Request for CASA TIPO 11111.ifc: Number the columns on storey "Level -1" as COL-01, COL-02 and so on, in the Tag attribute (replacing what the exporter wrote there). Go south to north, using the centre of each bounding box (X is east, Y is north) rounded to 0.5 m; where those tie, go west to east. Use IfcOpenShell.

First a look at what the model holds.

```python
import ifcopenshell
import ifcopenshell.util.element
import ifcopenshell.util.placement

model = ifcopenshell.open("CASA TIPO 11111.ifc")
print(model.schema)
storey = next(s for s in model.by_type("IfcBuildingStorey") if s.Name == "Level -1")
columns = [e for e in ifcopenshell.util.element.get_decomposition(storey) if e.is_a("IfcColumn")]
for e in sorted(columns, key=lambda e: e.id()):
    origin = ifcopenshell.util.placement.get_local_placement(e.ObjectPlacement)[:3, 3]
    print(e.id(), e.Tag, e.Name, origin.round(2) + 0.0, sep=" | ")
```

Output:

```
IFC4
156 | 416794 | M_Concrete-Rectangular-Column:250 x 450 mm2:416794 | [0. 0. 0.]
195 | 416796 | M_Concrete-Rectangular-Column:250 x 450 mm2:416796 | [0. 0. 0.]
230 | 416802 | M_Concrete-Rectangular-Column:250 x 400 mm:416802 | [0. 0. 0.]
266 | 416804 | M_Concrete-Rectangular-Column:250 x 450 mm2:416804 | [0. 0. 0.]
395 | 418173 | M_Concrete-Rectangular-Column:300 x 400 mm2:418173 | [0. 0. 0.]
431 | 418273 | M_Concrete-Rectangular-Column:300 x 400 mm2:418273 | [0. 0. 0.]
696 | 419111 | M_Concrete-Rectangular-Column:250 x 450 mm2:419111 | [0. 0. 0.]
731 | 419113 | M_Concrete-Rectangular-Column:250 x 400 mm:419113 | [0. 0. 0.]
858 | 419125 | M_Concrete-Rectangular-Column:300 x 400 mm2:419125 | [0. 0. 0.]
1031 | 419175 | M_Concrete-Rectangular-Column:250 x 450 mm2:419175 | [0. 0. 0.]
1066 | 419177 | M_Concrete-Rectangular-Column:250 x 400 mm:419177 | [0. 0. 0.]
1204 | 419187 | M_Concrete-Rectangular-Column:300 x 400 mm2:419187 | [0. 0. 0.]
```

```python
import ifcopenshell
import ifcopenshell.geom
import ifcopenshell.util.element
import ifcopenshell.util.shape

model = ifcopenshell.open("CASA TIPO 11111.ifc")
settings = ifcopenshell.geom.settings()
settings.set("use-world-coords", True)


def centre(element):
    shape = ifcopenshell.geom.create_shape(settings, element)
    return ifcopenshell.util.shape.get_bbox_centroid(shape.geometry)


storey = next(s for s in model.by_type("IfcBuildingStorey") if s.Name == "Level -1")
columns = [e for e in ifcopenshell.util.element.get_decomposition(storey) if e.is_a("IfcColumn")]

# Insertion points can sit at a corner or the storey origin, so sort by the geometry (in metres).
centres = {e: centre(e) for e in columns}
columns.sort(key=lambda e: (round(centres[e][1] / 0.5), centres[e][0]))

for i, e in enumerate(columns, start=1):
    number = f"COL-{i:02d}"
    e.Tag = number
    print(e.id(), number)

model.write("CASA TIPO 11111-out.ifc")
```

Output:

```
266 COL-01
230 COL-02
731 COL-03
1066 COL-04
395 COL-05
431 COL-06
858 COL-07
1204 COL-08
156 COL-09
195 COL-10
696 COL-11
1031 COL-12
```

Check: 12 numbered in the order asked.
